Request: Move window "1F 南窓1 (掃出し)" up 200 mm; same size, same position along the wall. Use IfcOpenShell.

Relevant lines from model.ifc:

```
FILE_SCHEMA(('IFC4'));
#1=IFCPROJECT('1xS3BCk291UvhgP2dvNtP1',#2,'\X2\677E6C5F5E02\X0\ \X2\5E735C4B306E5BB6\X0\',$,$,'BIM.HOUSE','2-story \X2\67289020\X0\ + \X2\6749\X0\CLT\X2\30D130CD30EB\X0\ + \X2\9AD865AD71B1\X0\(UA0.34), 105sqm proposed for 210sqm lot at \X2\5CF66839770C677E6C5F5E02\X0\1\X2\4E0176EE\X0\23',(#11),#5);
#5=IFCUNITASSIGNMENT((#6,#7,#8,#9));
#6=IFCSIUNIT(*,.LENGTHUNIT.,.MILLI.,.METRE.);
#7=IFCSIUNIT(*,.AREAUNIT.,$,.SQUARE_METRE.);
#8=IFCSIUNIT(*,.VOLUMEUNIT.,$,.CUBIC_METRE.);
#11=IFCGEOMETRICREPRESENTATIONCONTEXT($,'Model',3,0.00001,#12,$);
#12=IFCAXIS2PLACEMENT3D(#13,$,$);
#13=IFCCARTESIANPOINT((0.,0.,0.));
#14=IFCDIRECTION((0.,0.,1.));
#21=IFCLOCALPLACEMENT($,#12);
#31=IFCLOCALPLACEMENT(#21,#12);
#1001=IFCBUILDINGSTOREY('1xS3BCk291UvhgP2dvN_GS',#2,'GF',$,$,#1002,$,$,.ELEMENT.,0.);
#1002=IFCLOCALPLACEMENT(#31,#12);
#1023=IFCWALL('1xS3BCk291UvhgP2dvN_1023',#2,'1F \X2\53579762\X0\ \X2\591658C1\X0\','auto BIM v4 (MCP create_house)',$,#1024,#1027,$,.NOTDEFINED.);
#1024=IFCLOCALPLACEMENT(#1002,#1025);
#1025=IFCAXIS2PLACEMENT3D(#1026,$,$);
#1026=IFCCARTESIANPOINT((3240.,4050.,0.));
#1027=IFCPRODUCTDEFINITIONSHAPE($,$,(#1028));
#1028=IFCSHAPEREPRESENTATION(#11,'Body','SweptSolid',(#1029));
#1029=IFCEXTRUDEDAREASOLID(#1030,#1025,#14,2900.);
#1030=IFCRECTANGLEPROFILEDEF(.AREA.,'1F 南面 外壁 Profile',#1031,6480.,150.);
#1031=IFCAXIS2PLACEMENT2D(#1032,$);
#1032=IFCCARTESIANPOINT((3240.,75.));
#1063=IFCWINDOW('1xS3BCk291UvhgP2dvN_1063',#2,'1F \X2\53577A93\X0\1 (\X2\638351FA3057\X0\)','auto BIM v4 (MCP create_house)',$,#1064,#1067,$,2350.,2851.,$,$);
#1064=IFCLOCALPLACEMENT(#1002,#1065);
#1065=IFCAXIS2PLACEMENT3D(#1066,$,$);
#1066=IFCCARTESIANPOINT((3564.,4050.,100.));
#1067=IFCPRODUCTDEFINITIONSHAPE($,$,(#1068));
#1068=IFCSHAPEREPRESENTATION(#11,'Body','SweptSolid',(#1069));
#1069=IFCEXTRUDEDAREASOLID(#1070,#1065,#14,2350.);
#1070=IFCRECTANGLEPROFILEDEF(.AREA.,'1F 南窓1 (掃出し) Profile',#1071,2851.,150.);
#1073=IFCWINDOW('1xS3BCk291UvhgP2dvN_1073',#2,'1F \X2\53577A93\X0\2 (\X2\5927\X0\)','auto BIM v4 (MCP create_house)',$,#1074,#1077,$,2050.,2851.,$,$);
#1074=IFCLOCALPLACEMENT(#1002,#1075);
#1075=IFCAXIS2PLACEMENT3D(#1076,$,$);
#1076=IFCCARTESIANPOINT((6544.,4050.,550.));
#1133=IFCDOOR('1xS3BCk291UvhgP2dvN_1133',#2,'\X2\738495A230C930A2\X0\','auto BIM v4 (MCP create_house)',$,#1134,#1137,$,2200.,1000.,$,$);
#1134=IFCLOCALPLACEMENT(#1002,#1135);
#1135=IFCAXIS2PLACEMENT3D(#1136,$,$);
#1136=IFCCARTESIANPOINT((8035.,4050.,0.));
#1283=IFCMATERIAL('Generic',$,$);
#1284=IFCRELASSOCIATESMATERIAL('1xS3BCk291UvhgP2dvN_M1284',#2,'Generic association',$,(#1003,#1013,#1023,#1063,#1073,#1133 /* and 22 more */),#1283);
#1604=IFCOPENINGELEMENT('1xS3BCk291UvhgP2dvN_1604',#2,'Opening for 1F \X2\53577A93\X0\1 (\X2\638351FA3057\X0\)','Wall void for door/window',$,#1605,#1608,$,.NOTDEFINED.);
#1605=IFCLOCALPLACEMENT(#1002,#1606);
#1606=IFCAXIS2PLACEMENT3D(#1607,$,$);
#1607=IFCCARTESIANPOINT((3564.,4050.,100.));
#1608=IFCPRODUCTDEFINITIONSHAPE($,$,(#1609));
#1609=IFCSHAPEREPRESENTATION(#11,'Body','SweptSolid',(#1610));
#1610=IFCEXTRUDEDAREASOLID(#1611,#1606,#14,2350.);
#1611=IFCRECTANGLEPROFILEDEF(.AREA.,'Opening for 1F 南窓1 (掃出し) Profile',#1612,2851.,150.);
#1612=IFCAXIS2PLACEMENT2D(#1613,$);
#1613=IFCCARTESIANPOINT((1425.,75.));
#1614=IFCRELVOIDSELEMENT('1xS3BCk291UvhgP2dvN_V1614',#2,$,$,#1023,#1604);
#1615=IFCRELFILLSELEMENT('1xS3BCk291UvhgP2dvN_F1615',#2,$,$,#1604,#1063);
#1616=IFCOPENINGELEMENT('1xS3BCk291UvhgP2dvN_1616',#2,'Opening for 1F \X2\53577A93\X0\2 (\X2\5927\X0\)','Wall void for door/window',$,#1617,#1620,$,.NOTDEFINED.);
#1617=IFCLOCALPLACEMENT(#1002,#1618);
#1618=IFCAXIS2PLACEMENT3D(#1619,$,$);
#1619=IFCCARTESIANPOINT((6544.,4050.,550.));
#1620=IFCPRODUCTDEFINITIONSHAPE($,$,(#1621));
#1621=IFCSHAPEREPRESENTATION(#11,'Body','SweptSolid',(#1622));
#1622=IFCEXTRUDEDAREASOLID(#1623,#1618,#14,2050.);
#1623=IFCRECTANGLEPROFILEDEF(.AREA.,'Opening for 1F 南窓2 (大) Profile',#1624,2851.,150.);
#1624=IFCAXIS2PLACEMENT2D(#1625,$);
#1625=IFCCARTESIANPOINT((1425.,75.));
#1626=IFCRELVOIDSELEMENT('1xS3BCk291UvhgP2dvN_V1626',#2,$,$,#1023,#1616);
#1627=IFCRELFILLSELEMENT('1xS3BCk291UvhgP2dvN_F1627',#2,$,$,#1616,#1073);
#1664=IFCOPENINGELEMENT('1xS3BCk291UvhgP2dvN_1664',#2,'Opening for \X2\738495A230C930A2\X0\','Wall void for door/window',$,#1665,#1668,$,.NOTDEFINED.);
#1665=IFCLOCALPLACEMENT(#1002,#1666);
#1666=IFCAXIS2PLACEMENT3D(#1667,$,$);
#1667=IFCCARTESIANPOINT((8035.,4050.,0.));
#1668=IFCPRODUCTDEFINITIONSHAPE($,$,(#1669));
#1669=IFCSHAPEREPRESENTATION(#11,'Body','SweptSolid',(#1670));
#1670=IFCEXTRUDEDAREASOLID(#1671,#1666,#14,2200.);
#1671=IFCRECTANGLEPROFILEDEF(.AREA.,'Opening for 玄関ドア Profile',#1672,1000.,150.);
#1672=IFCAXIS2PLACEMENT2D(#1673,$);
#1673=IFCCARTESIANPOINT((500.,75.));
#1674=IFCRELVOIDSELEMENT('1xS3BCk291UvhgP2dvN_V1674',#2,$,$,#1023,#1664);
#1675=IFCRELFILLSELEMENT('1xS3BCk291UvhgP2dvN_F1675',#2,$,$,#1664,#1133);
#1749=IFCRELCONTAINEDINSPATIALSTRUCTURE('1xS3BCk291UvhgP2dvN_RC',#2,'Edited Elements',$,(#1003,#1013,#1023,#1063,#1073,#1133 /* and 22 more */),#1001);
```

```python
import numpy as np
import ifcopenshell
import ifcopenshell.api.geometry
import ifcopenshell.util.placement
import ifcopenshell.util.unit

model = ifcopenshell.open("model.ifc")
unit_scale = ifcopenshell.util.unit.calculate_unit_scale(model)

window = model.by_guid("1xS3BCk291UvhgP2dvN_1063")
opening = window.FillsVoids[0].RelatingOpeningElement
dz = 200.0

shift = np.array([0.0, 0.0, dz])
# The window is not placed relative to its opening, so move both.
for product in (opening, window):
    matrix = ifcopenshell.util.placement.get_local_placement(product.ObjectPlacement)
    matrix[:3, 3] += shift
    ifcopenshell.api.geometry.edit_object_placement(model, product=product, matrix=matrix, is_si=False)

print(f"moved by {dz * unit_scale:+.3f} m")

model.write("model_rev.ifc")
```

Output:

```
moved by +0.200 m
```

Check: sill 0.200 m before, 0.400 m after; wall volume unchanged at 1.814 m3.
